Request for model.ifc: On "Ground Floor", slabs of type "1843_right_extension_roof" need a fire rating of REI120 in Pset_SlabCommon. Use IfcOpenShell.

First a look at what the model holds.

```python
import ifcopenshell
import ifcopenshell.util.element

model = ifcopenshell.open("model.ifc")
print(model.schema)
storey = next(s for s in model.by_type("IfcBuildingStorey") if s.Name == "Ground Floor")
slabs = [e for e in ifcopenshell.util.element.get_decomposition(storey) if e.is_a("IfcSlab")]
seen = {}
for e in slabs:
    element_type = ifcopenshell.util.element.get_type(e)
    key = (element_type.Name if element_type != e and element_type else None, ifcopenshell.util.element.get_pset(e, "Pset_SlabCommon", "FireRating"))
    seen[key] = seen.get(key, 0) + 1
for (name, value), count in sorted(seen.items(), key=str):
    print(count, "x", name, "|", value)
```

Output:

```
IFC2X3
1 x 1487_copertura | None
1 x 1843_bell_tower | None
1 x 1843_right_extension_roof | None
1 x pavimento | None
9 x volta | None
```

```python
import ifcopenshell
import ifcopenshell.api.pset
import ifcopenshell.util.element

model = ifcopenshell.open("model.ifc")

storey = next(s for s in model.by_type("IfcBuildingStorey") if s.Name == "Ground Floor")
slabs = [e for e in ifcopenshell.util.element.get_decomposition(storey) if e.is_a("IfcSlab")]

count = 0
for e in slabs:
    element_type = ifcopenshell.util.element.get_type(e)
    if element_type in (None, e) or element_type.Name != "1843_right_extension_roof":
        continue
    # add_pset returns the element's existing set when there is one.
    pset = ifcopenshell.api.pset.add_pset(model, product=e, name="Pset_SlabCommon")
    ifcopenshell.api.pset.edit_pset(model, pset=pset, properties={"FireRating": "REI120"})
    count += 1

print(count, "slabs updated")

model.write("model-out.ifc")
```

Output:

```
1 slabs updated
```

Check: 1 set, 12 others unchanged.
